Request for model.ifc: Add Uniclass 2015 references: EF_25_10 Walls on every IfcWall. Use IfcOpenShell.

First a look at what the model holds.

```python
import ifcopenshell

model = ifcopenshell.open("model.ifc")
print(model.schema)
print("classifications:", [c.Name for c in model.by_type("IfcClassification")])
for ifc_class in ("IfcDoor", "IfcRoof", "IfcStair", "IfcWall", "IfcWindow"):
    print(ifc_class, len(model.by_type(ifc_class)))
```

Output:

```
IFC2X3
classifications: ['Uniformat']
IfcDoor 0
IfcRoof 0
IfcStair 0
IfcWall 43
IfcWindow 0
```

```python
import ifcopenshell
import ifcopenshell.api.classification

model = ifcopenshell.open("model.ifc")

# IFC2X3 requires Source and Edition and has no link from the project to the system.
system = model.create_entity("IfcClassification", Source="NBS", Edition="2015", Name="Uniclass 2015")

codes = {
    "IfcWall": ("EF_25_10", "Walls"),
}
for ifc_class, (code, name) in codes.items():
    products = model.by_type(ifc_class)
    ifcopenshell.api.classification.add_reference(
        model, products=products, classification=system, identification=code, name=name
    )
    print(code, len(products))

model.write("model_updated.ifc")
```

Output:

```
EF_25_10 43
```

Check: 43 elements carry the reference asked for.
